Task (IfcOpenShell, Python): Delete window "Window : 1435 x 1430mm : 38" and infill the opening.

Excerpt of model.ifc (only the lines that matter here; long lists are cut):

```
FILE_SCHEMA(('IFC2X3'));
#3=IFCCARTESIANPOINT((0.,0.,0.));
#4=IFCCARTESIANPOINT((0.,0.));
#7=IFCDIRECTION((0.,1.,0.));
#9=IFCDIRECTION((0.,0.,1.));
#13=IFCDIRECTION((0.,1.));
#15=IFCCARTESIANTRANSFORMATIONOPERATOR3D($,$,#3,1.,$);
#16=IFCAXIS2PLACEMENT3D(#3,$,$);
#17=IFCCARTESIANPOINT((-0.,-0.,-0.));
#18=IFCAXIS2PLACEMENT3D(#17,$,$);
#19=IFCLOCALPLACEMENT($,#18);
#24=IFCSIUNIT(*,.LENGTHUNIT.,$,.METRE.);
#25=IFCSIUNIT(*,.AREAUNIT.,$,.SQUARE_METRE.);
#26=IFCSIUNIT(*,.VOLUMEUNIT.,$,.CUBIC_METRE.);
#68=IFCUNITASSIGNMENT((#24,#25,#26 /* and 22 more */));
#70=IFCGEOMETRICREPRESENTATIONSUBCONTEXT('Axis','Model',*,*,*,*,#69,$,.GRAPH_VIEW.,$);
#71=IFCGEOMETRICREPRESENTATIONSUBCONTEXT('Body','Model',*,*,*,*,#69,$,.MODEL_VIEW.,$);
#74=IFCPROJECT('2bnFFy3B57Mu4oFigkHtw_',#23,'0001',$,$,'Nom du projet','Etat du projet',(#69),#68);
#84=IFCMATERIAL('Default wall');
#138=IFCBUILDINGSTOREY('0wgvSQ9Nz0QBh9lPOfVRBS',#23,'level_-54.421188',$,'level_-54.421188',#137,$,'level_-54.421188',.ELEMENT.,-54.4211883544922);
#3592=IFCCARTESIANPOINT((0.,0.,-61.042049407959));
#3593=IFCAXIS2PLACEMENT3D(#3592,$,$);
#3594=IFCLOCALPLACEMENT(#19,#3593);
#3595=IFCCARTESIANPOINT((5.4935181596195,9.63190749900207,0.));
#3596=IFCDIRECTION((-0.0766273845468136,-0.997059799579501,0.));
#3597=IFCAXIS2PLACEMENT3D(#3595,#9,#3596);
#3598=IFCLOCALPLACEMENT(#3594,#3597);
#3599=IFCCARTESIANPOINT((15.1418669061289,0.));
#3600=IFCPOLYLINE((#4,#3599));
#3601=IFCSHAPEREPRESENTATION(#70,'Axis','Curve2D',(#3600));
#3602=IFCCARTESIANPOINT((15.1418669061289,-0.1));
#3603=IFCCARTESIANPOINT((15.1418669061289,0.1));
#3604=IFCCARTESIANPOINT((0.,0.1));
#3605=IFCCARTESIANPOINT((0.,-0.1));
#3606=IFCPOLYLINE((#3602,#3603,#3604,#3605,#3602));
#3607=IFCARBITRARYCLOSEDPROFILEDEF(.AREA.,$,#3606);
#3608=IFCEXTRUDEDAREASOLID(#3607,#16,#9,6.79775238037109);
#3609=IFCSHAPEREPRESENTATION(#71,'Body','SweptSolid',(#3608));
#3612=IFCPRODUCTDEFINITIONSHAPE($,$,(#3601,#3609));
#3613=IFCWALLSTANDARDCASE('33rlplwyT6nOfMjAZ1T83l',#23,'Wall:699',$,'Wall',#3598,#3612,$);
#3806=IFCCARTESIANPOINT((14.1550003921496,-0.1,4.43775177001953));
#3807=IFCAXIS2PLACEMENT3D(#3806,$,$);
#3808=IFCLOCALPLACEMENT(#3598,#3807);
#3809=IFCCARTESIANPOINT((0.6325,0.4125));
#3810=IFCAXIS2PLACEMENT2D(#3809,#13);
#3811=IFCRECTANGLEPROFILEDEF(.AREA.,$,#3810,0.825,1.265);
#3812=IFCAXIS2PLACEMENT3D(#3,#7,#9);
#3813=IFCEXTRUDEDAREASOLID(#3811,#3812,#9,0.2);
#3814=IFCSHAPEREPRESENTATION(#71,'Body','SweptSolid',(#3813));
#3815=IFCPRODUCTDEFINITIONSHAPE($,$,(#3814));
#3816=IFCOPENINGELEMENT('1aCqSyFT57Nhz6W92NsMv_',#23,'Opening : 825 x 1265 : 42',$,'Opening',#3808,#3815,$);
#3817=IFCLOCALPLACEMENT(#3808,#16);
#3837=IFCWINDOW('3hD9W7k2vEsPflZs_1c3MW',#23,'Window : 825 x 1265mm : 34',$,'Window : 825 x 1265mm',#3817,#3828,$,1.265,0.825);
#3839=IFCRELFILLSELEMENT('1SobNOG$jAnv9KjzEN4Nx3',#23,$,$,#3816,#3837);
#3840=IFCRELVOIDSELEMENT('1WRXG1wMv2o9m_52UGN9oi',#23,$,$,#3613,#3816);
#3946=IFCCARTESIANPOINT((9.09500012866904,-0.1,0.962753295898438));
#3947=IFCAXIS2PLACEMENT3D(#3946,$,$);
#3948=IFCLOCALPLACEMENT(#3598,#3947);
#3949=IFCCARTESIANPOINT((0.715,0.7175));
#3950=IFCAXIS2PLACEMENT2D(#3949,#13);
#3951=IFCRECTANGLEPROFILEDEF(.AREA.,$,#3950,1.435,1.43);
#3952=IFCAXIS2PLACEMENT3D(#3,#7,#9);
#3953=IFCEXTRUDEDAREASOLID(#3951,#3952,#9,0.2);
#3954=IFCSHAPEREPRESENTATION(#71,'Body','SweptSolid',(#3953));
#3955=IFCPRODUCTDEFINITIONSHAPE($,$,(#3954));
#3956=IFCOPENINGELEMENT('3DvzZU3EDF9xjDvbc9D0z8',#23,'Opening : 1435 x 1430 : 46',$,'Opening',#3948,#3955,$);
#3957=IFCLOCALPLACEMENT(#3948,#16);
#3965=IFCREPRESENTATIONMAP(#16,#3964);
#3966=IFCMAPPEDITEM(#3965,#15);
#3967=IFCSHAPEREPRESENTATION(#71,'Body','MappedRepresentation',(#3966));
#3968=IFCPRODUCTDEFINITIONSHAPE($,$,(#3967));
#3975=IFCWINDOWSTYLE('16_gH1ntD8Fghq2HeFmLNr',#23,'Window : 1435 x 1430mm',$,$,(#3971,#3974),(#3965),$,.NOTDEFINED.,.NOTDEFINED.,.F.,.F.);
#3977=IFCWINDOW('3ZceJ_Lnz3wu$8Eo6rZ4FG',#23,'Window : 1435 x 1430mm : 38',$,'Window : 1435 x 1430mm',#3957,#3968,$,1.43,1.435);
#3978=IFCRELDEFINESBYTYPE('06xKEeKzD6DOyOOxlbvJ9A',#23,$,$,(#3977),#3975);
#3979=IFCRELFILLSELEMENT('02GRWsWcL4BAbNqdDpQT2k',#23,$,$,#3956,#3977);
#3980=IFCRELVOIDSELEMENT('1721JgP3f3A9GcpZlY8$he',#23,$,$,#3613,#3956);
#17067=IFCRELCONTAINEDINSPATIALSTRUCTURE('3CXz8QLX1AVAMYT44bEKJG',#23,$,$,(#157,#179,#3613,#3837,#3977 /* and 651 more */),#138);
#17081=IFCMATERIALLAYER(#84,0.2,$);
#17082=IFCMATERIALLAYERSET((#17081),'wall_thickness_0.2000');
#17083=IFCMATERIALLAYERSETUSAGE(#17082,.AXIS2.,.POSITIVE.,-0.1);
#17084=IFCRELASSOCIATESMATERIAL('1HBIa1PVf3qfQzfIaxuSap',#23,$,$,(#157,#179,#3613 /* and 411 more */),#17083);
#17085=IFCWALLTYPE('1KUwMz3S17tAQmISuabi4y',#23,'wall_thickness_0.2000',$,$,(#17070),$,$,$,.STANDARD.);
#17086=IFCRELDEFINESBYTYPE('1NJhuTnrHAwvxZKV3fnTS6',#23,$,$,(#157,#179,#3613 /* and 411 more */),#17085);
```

```python
import ifcopenshell
import ifcopenshell.api.feature
import ifcopenshell.api.root
import ifcopenshell.geom
import ifcopenshell.util.shape

model = ifcopenshell.open("model.ifc")
settings = ifcopenshell.geom.settings()


def volume(element):
    """Net volume in cubic metres, openings subtracted."""
    shape = ifcopenshell.geom.create_shape(settings, element)
    return ifcopenshell.util.shape.get_volume(shape.geometry)


window = model.by_guid("3ZceJ_Lnz3wu$8Eo6rZ4FG")
opening = window.FillsVoids[0].RelatingOpeningElement
wall = opening.VoidsElements[0].RelatingBuildingElement
before = volume(wall)

ifcopenshell.api.root.remove_product(model, product=window)
ifcopenshell.api.feature.remove_feature(model, feature=opening)

after = volume(wall)

print(f"wall volume {before:.3f} -> {after:.3f} m3")

model.write("model_v2.ifc")
```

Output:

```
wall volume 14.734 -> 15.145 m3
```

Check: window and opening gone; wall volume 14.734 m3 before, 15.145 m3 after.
